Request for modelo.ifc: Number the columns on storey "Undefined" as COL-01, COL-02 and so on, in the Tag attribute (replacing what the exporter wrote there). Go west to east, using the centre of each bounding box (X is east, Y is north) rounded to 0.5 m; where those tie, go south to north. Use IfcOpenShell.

First a look at what the model holds.

```python
import ifcopenshell
import ifcopenshell.util.element
import ifcopenshell.util.placement

model = ifcopenshell.open("modelo.ifc")
print(model.schema)
storey = next(s for s in model.by_type("IfcBuildingStorey") if s.Name == "Undefined")
columns = [e for e in ifcopenshell.util.element.get_decomposition(storey) if e.is_a("IfcColumn")]
for e in sorted(columns, key=lambda e: e.id()):
    origin = ifcopenshell.util.placement.get_local_placement(e.ObjectPlacement)[:3, 3]
    print(e.id(), e.Tag, e.Name, origin.round(2) + 0.0, sep=" | ")
```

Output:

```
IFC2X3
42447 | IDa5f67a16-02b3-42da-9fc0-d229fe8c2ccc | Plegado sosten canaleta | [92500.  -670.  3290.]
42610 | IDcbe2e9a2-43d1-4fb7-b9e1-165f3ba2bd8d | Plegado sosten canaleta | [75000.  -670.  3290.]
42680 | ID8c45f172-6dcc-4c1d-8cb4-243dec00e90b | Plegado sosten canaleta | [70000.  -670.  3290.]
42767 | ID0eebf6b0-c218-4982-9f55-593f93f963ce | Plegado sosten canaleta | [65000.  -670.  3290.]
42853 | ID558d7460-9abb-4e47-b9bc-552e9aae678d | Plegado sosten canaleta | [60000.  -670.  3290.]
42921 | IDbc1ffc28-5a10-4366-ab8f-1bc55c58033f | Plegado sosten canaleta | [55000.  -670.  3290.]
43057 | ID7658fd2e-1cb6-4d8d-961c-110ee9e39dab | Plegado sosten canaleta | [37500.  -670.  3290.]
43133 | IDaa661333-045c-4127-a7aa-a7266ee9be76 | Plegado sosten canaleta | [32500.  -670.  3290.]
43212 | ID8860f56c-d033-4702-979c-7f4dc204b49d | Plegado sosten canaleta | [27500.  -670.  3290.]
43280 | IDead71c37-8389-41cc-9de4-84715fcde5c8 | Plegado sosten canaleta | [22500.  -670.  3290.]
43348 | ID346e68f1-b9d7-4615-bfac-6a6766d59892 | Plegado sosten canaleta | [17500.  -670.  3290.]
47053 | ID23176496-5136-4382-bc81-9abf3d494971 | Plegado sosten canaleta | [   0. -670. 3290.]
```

```python
import ifcopenshell
import ifcopenshell.geom
import ifcopenshell.util.element
import ifcopenshell.util.shape

model = ifcopenshell.open("modelo.ifc")
settings = ifcopenshell.geom.settings()
settings.set("use-world-coords", True)


def centre(element):
    shape = ifcopenshell.geom.create_shape(settings, element)
    return ifcopenshell.util.shape.get_bbox_centroid(shape.geometry)


storey = next(s for s in model.by_type("IfcBuildingStorey") if s.Name == "Undefined")
columns = [e for e in ifcopenshell.util.element.get_decomposition(storey) if e.is_a("IfcColumn")]

# Insertion points can sit at a corner or the storey origin, so sort by the geometry (in metres).
centres = {e: centre(e) for e in columns}
columns.sort(key=lambda e: (round(centres[e][0] / 0.5), centres[e][1]))

for i, e in enumerate(columns, start=1):
    number = f"COL-{i:02d}"
    e.Tag = number
    print(e.id(), number)

model.write("modelo-out.ifc")
```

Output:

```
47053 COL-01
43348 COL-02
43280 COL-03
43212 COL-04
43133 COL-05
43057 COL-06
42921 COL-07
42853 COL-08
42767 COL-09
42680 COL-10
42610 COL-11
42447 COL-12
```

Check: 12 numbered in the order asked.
